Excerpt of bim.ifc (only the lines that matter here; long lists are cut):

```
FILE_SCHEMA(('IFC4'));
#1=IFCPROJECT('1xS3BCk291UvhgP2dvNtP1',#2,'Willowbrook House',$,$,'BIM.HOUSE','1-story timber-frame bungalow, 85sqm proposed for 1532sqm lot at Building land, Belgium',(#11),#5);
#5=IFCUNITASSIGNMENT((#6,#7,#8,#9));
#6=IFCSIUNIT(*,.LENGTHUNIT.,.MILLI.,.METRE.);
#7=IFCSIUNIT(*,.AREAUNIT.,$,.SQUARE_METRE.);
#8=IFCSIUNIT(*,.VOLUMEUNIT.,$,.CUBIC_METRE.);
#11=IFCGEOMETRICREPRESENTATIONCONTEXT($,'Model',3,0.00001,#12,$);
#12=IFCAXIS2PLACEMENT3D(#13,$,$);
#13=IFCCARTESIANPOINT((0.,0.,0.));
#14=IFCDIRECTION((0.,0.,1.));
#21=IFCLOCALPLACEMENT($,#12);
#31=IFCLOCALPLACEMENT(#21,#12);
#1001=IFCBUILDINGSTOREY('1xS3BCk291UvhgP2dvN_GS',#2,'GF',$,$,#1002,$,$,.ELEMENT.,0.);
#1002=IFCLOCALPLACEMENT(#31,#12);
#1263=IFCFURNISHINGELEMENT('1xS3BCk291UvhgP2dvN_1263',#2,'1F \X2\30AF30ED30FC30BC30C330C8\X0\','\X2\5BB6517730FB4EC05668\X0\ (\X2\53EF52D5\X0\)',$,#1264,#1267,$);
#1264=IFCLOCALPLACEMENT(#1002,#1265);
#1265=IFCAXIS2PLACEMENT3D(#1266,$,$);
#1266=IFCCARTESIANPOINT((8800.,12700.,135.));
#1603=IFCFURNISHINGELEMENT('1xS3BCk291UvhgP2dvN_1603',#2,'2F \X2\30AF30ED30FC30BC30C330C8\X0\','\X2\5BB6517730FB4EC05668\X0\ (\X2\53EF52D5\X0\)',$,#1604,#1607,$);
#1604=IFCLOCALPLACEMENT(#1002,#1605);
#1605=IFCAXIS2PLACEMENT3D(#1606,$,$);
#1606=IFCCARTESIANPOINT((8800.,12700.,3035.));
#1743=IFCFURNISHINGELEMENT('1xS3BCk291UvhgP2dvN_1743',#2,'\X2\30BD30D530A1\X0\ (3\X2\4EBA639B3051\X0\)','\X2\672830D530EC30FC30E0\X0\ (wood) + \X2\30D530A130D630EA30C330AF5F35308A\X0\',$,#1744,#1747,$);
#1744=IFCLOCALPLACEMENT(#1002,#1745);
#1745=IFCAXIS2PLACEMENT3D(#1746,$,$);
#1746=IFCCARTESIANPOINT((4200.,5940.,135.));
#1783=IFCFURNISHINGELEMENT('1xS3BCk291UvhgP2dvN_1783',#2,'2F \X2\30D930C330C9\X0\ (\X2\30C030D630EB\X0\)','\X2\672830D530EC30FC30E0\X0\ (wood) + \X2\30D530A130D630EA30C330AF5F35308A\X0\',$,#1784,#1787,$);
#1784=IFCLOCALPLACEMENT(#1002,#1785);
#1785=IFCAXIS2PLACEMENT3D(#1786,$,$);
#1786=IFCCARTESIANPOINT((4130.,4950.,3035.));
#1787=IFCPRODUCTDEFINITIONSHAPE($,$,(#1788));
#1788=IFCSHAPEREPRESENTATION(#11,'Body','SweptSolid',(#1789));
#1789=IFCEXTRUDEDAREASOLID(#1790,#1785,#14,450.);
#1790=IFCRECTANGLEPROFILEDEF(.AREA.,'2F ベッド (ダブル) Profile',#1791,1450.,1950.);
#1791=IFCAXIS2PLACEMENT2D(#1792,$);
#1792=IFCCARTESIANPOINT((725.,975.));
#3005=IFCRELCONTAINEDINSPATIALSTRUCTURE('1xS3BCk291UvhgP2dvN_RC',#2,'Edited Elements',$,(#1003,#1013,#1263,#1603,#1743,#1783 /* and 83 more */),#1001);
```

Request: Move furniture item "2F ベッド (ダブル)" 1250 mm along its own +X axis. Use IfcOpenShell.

```python
import ifcopenshell
import ifcopenshell.api.geometry
import ifcopenshell.util.placement

model = ifcopenshell.open("bim.ifc")

item = model.by_id(1783)
matrix = ifcopenshell.util.placement.get_local_placement(item.ObjectPlacement)
matrix[:3, 3] += matrix[:3, 0] * 1250.0
ifcopenshell.api.geometry.edit_object_placement(model, product=item, matrix=matrix, is_si=False)

print(ifcopenshell.util.placement.get_local_placement(item.ObjectPlacement).round(3) + 0.0)

model.write("bim_edited.ifc")
```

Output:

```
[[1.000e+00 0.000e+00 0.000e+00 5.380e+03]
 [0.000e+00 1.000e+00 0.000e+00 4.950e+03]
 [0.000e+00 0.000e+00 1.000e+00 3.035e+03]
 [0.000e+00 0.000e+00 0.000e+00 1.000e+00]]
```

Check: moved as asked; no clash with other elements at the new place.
